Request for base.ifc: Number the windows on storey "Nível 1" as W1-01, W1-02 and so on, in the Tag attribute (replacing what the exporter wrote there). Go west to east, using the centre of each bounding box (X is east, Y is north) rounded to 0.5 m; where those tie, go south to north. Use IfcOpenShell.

First a look at what the model holds.

```python
import ifcopenshell
import ifcopenshell.util.element
import ifcopenshell.util.placement

model = ifcopenshell.open("base.ifc")
print(model.schema)
storey = next(s for s in model.by_type("IfcBuildingStorey") if s.Name == "Nível 1")
windows = [e for e in ifcopenshell.util.element.get_decomposition(storey) if e.is_a("IfcWindow")]
for e in sorted(windows, key=lambda e: e.id()):
    origin = ifcopenshell.util.placement.get_local_placement(e.ObjectPlacement)[:3, 3]
    print(e.id(), e.Tag, e.Name, origin.round(2) + 0.0, sep=" | ")
```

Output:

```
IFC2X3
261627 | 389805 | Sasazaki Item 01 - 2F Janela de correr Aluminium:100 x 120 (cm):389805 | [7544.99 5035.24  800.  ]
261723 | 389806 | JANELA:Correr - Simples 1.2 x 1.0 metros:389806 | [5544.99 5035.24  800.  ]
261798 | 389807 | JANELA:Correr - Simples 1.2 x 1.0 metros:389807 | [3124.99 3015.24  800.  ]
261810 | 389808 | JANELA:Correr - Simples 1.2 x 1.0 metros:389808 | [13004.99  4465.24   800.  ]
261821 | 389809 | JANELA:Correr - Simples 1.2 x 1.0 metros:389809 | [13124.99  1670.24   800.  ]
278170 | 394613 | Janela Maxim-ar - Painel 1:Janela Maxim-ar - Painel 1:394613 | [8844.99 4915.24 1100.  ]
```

```python
import ifcopenshell
import ifcopenshell.geom
import ifcopenshell.util.element
import ifcopenshell.util.shape

model = ifcopenshell.open("base.ifc")
settings = ifcopenshell.geom.settings()
settings.set("use-world-coords", True)


def centre(element):
    shape = ifcopenshell.geom.create_shape(settings, element)
    return ifcopenshell.util.shape.get_bbox_centroid(shape.geometry)


storey = next(s for s in model.by_type("IfcBuildingStorey") if s.Name == "Nível 1")
windows = [e for e in ifcopenshell.util.element.get_decomposition(storey) if e.is_a("IfcWindow")]

# Insertion points can sit at a corner or the storey origin, so sort by the geometry (in metres).
centres = {e: centre(e) for e in windows}
windows.sort(key=lambda e: (round(centres[e][0] / 0.5), centres[e][1]))

for i, e in enumerate(windows, start=1):
    number = f"W1-{i:02d}"
    e.Tag = number
    print(e.id(), number)

model.write("base_edited.ifc")
```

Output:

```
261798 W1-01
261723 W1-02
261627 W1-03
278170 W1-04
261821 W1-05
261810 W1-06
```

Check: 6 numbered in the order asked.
